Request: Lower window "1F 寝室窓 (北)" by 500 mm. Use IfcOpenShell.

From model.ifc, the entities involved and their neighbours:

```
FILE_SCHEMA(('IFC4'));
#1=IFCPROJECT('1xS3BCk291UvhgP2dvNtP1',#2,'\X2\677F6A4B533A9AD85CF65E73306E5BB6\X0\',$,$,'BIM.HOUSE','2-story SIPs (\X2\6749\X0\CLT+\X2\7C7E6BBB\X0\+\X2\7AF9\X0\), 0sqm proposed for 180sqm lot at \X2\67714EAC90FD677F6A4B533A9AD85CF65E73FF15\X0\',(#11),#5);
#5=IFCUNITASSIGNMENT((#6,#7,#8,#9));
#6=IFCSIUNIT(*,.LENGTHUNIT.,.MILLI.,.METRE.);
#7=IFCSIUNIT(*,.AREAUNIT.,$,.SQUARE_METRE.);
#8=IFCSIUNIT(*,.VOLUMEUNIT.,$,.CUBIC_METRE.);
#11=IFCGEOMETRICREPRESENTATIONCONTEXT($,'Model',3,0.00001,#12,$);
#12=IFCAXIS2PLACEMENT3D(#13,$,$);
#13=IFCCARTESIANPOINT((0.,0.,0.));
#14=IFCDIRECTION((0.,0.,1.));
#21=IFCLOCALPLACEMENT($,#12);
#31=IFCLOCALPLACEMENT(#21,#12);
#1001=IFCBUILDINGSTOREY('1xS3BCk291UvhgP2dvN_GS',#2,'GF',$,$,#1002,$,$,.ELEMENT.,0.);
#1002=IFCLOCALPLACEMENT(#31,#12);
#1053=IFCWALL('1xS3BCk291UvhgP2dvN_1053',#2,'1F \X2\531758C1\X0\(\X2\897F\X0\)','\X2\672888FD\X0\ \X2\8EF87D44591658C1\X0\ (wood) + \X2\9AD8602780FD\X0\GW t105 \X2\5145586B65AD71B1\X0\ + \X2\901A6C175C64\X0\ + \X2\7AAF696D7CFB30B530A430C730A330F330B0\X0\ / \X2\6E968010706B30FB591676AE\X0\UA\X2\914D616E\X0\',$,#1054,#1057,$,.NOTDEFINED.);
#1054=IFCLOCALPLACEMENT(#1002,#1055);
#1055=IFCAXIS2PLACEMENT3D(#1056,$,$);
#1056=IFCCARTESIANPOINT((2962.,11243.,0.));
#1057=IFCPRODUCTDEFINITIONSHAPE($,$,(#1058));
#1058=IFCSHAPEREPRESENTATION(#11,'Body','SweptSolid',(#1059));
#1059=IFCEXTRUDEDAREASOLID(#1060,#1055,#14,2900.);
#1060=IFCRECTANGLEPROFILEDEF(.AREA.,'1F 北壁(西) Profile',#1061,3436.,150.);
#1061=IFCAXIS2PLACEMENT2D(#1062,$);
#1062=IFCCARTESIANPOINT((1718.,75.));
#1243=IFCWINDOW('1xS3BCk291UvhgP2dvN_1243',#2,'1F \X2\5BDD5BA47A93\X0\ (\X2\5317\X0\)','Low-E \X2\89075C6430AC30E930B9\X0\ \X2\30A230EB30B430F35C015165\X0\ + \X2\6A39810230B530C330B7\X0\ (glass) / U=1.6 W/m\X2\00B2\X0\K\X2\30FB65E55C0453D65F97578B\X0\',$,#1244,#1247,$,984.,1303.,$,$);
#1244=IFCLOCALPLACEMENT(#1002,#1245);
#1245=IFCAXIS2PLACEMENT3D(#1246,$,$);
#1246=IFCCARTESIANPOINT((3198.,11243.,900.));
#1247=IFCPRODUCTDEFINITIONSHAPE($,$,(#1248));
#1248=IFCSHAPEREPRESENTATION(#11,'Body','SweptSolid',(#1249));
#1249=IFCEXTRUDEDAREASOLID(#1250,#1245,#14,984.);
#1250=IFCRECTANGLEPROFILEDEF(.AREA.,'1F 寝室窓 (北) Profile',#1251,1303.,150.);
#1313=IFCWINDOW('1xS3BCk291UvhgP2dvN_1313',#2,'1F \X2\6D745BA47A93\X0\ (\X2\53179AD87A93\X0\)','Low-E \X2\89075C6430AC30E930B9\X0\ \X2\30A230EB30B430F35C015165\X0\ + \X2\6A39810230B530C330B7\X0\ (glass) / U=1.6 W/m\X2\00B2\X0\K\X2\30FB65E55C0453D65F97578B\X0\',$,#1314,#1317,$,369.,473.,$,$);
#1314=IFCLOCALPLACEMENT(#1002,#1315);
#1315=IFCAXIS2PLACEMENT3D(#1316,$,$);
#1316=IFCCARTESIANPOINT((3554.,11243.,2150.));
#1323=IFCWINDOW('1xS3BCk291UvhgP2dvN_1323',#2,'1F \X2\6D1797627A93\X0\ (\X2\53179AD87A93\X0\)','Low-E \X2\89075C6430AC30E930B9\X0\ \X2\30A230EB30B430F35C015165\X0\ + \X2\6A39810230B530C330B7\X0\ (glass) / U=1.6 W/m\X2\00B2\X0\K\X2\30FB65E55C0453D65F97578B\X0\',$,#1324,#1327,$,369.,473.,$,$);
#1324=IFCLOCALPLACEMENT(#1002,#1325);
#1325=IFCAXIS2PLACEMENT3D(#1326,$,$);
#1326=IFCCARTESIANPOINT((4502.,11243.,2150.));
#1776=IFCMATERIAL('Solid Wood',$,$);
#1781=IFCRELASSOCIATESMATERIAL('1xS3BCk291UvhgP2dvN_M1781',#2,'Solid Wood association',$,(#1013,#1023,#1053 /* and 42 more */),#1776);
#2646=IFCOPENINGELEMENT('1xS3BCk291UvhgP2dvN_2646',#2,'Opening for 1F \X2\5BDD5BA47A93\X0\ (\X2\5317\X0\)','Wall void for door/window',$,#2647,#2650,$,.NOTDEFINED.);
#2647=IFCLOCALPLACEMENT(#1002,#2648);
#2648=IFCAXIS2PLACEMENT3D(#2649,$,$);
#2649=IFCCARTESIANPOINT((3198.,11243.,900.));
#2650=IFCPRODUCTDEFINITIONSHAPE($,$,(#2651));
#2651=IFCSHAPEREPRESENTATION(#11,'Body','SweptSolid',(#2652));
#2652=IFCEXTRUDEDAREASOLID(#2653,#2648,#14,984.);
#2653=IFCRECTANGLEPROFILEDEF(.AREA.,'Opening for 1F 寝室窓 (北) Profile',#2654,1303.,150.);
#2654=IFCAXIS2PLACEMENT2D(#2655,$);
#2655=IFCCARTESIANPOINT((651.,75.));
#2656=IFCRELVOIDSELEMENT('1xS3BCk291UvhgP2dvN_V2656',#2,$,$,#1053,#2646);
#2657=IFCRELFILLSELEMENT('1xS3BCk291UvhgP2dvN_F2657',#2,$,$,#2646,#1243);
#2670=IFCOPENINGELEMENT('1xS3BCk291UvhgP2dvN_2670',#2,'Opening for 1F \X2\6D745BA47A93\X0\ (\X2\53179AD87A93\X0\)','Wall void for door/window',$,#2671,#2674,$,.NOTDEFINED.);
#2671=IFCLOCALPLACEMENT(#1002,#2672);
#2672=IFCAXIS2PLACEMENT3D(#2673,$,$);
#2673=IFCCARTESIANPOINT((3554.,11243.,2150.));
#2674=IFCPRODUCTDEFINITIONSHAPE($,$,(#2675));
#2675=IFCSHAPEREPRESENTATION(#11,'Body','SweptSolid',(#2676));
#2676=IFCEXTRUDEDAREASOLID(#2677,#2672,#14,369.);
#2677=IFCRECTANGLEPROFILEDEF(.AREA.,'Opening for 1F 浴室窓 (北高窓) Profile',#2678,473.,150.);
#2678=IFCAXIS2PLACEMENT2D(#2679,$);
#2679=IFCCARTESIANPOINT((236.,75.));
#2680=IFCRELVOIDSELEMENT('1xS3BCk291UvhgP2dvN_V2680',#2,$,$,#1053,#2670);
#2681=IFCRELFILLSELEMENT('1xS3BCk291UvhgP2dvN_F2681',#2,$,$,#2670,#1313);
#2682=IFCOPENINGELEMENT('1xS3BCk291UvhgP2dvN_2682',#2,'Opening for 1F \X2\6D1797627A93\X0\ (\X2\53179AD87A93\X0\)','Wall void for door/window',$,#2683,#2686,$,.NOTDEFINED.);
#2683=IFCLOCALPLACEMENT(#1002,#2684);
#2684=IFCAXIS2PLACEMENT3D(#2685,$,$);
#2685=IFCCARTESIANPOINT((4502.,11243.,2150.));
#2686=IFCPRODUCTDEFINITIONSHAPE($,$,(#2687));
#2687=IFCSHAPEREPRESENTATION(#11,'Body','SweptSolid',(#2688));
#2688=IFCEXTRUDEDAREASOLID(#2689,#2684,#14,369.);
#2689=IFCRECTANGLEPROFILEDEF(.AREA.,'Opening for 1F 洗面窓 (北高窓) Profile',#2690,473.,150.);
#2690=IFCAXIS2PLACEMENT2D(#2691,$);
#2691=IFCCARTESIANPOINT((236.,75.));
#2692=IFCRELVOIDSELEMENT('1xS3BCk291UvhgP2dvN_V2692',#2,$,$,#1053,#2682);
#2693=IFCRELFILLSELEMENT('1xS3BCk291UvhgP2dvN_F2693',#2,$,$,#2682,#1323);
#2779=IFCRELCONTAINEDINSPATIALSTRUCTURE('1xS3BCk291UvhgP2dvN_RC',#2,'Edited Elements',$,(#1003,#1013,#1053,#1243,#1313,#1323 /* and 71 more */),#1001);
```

```python
import numpy as np
import ifcopenshell
import ifcopenshell.api.geometry
import ifcopenshell.util.placement
import ifcopenshell.util.unit

model = ifcopenshell.open("model.ifc")
unit_scale = ifcopenshell.util.unit.calculate_unit_scale(model)

window = model.by_guid("1xS3BCk291UvhgP2dvN_1243")
opening = window.FillsVoids[0].RelatingOpeningElement
dz = -0.5 / unit_scale

shift = np.array([0.0, 0.0, dz])
# The window is not placed relative to its opening, so move both.
for product in (opening, window):
    matrix = ifcopenshell.util.placement.get_local_placement(product.ObjectPlacement)
    matrix[:3, 3] += shift
    ifcopenshell.api.geometry.edit_object_placement(model, product=product, matrix=matrix, is_si=False)

print(f"moved by {dz * unit_scale:+.3f} m")

model.write("model_edited.ifc")
```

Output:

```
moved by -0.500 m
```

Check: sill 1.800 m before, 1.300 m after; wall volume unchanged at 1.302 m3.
